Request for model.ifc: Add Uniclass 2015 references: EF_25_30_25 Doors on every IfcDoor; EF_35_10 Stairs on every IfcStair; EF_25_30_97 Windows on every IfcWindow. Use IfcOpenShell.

First a look at what the model holds.

```python
import ifcopenshell

model = ifcopenshell.open("model.ifc")
print(model.schema)
print("classifications:", [c.Name for c in model.by_type("IfcClassification")])
for ifc_class in ("IfcDoor", "IfcRoof", "IfcStair", "IfcWall", "IfcWindow"):
    print(ifc_class, len(model.by_type(ifc_class)))
```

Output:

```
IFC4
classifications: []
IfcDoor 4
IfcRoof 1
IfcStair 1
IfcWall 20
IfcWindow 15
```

```python
import ifcopenshell
import ifcopenshell.api.classification

model = ifcopenshell.open("model.ifc")

system = ifcopenshell.api.classification.add_classification(model, classification="Uniclass 2015")

codes = {
    "IfcDoor": ("EF_25_30_25", "Doors"),
    "IfcStair": ("EF_35_10", "Stairs"),
    "IfcWindow": ("EF_25_30_97", "Windows"),
}
for ifc_class, (code, name) in codes.items():
    products = model.by_type(ifc_class)
    ifcopenshell.api.classification.add_reference(
        model, products=products, classification=system, identification=code, name=name
    )
    print(code, len(products))

model.write("model-out.ifc")
```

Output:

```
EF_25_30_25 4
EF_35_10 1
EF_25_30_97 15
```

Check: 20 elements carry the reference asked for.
